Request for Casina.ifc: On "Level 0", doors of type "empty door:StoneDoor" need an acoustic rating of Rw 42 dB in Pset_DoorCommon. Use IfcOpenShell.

First a look at what the model holds.

```python
import ifcopenshell
import ifcopenshell.util.element

model = ifcopenshell.open("Casina.ifc")
print(model.schema)
storey = next(s for s in model.by_type("IfcBuildingStorey") if s.Name == "Level 0")
doors = [e for e in ifcopenshell.util.element.get_decomposition(storey) if e.is_a("IfcDoor")]
seen = {}
for e in doors:
    element_type = ifcopenshell.util.element.get_type(e)
    key = (element_type.Name if element_type != e and element_type else None, ifcopenshell.util.element.get_pset(e, "Pset_DoorCommon", "AcousticRating"))
    seen[key] = seen.get(key, 0) + 1
for (name, value), count in sorted(seen.items(), key=str):
    print(count, "x", name, "|", value)
```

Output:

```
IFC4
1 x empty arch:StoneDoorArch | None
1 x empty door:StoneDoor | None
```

```python
import ifcopenshell
import ifcopenshell.api.pset
import ifcopenshell.util.element

model = ifcopenshell.open("Casina.ifc")

storey = next(s for s in model.by_type("IfcBuildingStorey") if s.Name == "Level 0")
doors = [e for e in ifcopenshell.util.element.get_decomposition(storey) if e.is_a("IfcDoor")]

count = 0
for e in doors:
    element_type = ifcopenshell.util.element.get_type(e)
    if element_type in (None, e) or element_type.Name != "empty door:StoneDoor":
        continue
    # add_pset returns the element's existing set when there is one.
    pset = ifcopenshell.api.pset.add_pset(model, product=e, name="Pset_DoorCommon")
    ifcopenshell.api.pset.edit_pset(model, pset=pset, properties={"AcousticRating": "Rw 42 dB"})
    count += 1

print(count, "doors updated")

model.write("Casina_v2.ifc")
```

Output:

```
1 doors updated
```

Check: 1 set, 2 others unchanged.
